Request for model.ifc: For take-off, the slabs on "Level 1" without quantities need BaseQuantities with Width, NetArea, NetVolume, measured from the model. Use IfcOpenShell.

First a look at what the model holds.

```python
import ifcopenshell
import ifcopenshell.util.element
import ifcopenshell.util.unit

model = ifcopenshell.open("model.ifc")
print(model.schema)
for unit_type in ("LENGTHUNIT", "AREAUNIT", "VOLUMEUNIT"):
    print(unit_type, ifcopenshell.util.unit.calculate_unit_scale(model, unit_type))
storey = next(s for s in model.by_type("IfcBuildingStorey") if s.Name == "Level 1")
slabs = [e for e in ifcopenshell.util.element.get_decomposition(storey) if e.is_a("IfcSlab")]
for e in sorted(slabs, key=lambda e: e.id()):
    print(e.id(), e.is_a(), e.Name, list(ifcopenshell.util.element.get_psets(e, qtos_only=True)), sep=" | ")
```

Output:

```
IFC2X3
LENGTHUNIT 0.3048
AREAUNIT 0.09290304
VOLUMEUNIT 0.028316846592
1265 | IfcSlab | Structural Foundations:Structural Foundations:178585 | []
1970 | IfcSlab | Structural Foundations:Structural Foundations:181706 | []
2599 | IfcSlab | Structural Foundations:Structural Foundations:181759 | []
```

```python
import ifcopenshell
import ifcopenshell.api.pset
import ifcopenshell.geom
import ifcopenshell.util.element
import ifcopenshell.util.shape
import ifcopenshell.util.unit

model = ifcopenshell.open("model.ifc")
unit_scale = ifcopenshell.util.unit.calculate_unit_scale(model)
area_scale = ifcopenshell.util.unit.calculate_unit_scale(model, "AREAUNIT")
volume_scale = ifcopenshell.util.unit.calculate_unit_scale(model, "VOLUMEUNIT")
settings = ifcopenshell.geom.settings()

storey = next(s for s in model.by_type("IfcBuildingStorey") if s.Name == "Level 1")
slabs = [e for e in ifcopenshell.util.element.get_decomposition(storey) if e.is_a("IfcSlab")]

for e in sorted(slabs, key=lambda e: e.id()):
    if ifcopenshell.util.element.get_psets(e, qtos_only=True, should_inherit=False):
        continue
    # Geometry comes back in metres, in the element's own axes.
    shape = ifcopenshell.geom.create_shape(settings, e)
    values = {
        "Width": ifcopenshell.util.shape.get_z(shape.geometry) / unit_scale,
        "NetArea": ifcopenshell.util.shape.get_footprint_area(shape.geometry) / area_scale,
        "NetVolume": ifcopenshell.util.shape.get_volume(shape.geometry) / volume_scale,
    }
    qto = ifcopenshell.api.pset.add_qto(model, product=e, name="BaseQuantities")
    ifcopenshell.api.pset.edit_qto(model, qto=qto, properties=values)
    print(e.id(), {k: round(v, 3) for k, v in values.items()})

model.write("model_v2.ifc")
```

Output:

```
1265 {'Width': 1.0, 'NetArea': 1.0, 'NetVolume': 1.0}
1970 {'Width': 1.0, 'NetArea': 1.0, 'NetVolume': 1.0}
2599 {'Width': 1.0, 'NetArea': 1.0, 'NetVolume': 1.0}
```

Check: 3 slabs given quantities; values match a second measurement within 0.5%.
